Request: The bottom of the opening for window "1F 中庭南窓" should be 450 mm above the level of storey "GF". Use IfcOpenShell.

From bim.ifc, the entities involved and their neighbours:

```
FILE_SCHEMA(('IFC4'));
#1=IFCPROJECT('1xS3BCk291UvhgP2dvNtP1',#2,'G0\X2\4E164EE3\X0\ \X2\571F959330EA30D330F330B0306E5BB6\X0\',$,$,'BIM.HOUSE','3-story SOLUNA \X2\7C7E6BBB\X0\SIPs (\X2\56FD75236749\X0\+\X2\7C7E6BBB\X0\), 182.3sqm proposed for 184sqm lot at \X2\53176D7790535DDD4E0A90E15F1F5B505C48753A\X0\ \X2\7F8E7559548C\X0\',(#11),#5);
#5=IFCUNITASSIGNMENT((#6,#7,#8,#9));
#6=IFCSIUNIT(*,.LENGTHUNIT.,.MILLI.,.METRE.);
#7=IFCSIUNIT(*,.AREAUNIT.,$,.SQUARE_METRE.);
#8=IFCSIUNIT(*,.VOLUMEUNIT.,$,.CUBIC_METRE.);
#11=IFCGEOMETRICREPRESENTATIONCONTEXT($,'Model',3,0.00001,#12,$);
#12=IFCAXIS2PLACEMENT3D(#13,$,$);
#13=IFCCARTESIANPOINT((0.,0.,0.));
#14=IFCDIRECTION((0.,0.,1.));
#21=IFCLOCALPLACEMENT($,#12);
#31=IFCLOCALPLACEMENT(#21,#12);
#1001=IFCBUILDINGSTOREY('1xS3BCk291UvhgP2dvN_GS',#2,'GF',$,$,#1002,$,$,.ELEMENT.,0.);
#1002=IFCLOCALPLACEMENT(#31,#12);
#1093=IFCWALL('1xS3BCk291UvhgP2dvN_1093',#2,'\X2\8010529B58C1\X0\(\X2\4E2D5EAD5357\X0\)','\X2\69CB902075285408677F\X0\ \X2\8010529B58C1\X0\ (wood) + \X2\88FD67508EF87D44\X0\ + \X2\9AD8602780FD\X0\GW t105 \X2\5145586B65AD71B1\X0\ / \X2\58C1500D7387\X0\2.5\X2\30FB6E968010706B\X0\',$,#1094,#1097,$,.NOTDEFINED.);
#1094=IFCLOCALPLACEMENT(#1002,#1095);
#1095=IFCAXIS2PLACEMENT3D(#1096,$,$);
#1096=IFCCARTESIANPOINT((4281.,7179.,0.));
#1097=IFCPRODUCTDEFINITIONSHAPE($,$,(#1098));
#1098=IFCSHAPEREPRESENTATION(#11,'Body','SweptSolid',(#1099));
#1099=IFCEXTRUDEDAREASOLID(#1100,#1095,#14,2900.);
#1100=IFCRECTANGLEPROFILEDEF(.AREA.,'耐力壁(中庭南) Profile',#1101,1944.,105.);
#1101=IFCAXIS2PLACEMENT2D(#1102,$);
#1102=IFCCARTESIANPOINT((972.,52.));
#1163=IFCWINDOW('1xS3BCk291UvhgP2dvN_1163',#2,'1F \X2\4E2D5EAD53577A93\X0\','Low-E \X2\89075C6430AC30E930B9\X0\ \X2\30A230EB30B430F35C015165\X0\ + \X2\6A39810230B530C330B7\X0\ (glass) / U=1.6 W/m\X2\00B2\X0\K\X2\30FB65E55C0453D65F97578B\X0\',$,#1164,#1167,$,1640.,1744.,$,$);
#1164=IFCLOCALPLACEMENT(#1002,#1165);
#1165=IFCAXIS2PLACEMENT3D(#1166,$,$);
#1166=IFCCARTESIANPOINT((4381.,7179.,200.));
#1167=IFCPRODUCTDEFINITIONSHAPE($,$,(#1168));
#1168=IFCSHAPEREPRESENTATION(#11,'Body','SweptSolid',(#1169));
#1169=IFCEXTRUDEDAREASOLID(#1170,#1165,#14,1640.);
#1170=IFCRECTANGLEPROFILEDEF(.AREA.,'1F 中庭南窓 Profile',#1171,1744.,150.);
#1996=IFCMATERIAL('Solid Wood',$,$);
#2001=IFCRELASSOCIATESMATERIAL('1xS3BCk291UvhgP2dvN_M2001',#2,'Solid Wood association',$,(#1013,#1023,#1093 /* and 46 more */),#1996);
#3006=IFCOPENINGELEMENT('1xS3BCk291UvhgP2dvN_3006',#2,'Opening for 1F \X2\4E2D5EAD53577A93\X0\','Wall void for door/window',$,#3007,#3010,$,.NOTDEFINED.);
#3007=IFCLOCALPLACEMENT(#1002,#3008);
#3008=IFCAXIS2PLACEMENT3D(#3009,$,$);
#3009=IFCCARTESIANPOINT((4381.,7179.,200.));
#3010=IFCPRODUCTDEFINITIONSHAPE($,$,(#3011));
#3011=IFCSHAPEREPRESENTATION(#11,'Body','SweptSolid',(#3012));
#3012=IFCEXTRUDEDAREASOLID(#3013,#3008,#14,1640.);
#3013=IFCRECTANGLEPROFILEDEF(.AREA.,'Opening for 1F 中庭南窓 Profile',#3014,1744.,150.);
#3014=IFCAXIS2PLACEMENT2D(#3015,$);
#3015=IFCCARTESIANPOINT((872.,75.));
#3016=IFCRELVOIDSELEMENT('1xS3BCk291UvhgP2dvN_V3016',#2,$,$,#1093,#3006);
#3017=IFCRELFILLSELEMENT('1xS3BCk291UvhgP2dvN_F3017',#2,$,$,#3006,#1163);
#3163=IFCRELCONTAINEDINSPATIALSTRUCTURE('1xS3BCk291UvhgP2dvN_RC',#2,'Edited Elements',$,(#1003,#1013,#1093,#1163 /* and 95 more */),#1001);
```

```python
import numpy as np
import ifcopenshell
import ifcopenshell.api.geometry
import ifcopenshell.geom
import ifcopenshell.util.element
import ifcopenshell.util.placement
import ifcopenshell.util.shape
import ifcopenshell.util.unit

model = ifcopenshell.open("bim.ifc")
unit_scale = ifcopenshell.util.unit.calculate_unit_scale(model)

window = model.by_guid("1xS3BCk291UvhgP2dvN_1163")
opening = window.FillsVoids[0].RelatingOpeningElement
storey = ifcopenshell.util.element.get_container(window, ifc_class="IfcBuildingStorey")
level = ifcopenshell.util.placement.get_local_placement(storey.ObjectPlacement)[2, 3]

# The opening's origin need not be at the sill, so measure its lowest point.
shape = ifcopenshell.geom.create_shape(ifcopenshell.geom.settings(), opening)
bottom = ifcopenshell.util.shape.get_shape_bottom_elevation(shape, shape.geometry) / unit_scale
dz = level + 0.45 / unit_scale - bottom

shift = np.array([0.0, 0.0, dz])
# The window is not placed relative to its opening, so move both.
for product in (opening, window):
    matrix = ifcopenshell.util.placement.get_local_placement(product.ObjectPlacement)
    matrix[:3, 3] += shift
    ifcopenshell.api.geometry.edit_object_placement(model, product=product, matrix=matrix, is_si=False)

print(f"moved by {dz * unit_scale:+.3f} m")

model.write("bim_v2.ifc")
```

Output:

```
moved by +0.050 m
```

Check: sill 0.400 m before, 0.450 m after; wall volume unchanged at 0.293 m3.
